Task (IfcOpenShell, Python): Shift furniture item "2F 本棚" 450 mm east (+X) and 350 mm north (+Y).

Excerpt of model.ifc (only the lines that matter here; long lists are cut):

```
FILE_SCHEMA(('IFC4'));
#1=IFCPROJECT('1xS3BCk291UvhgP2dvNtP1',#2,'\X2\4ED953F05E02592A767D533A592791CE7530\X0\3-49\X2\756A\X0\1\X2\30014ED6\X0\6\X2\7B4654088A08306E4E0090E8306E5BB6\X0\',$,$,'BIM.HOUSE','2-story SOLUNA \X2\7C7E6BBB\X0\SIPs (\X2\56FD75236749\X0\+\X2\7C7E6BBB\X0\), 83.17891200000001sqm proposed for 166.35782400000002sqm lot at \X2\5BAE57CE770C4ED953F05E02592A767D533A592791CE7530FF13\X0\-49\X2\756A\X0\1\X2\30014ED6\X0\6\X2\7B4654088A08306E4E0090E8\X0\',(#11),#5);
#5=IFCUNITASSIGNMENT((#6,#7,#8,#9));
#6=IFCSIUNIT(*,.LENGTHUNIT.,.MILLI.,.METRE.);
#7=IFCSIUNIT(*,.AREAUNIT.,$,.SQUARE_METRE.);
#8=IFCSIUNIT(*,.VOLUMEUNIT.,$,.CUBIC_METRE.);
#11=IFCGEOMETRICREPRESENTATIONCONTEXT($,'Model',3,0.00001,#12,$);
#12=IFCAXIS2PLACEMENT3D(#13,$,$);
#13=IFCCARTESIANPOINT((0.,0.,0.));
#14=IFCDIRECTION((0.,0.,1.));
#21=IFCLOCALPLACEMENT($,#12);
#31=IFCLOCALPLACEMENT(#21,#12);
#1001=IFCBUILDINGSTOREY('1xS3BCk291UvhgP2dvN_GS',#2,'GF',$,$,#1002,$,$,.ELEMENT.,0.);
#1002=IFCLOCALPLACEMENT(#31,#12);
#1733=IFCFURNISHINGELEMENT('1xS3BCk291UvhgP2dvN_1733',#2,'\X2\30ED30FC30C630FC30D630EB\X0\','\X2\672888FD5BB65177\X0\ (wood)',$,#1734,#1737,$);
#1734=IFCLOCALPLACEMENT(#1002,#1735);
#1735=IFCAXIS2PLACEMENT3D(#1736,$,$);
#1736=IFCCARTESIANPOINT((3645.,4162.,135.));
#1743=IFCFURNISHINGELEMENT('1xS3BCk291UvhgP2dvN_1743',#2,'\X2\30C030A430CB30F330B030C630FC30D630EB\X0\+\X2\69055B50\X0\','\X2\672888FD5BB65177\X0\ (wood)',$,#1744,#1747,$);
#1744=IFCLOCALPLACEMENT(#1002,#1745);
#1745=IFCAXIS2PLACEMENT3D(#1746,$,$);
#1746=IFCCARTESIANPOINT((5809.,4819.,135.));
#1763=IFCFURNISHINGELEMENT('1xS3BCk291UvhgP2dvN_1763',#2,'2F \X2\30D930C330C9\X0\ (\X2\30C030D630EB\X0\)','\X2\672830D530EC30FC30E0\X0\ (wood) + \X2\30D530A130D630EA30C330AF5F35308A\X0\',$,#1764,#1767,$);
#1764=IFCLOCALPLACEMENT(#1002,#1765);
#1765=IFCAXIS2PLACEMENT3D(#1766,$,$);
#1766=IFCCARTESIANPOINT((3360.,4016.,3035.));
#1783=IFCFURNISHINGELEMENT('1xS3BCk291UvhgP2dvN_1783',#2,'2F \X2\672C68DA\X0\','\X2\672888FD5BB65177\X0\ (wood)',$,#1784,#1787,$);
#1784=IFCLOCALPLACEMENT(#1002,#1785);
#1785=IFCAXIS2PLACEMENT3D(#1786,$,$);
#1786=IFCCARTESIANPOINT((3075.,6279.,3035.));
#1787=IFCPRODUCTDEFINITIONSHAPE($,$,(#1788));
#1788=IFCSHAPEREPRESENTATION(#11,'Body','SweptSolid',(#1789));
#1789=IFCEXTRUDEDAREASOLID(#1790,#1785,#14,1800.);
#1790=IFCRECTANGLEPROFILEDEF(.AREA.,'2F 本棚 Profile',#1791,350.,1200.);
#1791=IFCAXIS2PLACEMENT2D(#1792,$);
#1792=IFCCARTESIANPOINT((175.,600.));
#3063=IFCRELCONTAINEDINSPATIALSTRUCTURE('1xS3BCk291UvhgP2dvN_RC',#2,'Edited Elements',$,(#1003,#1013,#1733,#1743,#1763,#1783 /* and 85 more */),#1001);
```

```python
import ifcopenshell
import ifcopenshell.api.geometry
import ifcopenshell.util.placement
import ifcopenshell.util.unit

model = ifcopenshell.open("model.ifc")
unit_scale = ifcopenshell.util.unit.calculate_unit_scale(model)

item = model.by_guid("1xS3BCk291UvhgP2dvN_1783")
matrix = ifcopenshell.util.placement.get_local_placement(item.ObjectPlacement)
matrix[0, 3] += 0.45 / unit_scale
matrix[1, 3] += 0.35 / unit_scale
ifcopenshell.api.geometry.edit_object_placement(model, product=item, matrix=matrix, is_si=False)

print(ifcopenshell.util.placement.get_local_placement(item.ObjectPlacement).round(3) + 0.0)

model.write("model_edited.ifc")
```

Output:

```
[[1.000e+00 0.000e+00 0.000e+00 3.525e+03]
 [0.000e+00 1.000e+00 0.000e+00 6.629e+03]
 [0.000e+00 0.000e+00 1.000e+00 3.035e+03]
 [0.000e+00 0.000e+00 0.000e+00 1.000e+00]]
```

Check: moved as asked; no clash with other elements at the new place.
